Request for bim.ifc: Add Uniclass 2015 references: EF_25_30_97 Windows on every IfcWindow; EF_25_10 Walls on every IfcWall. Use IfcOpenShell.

First a look at what the model holds.

```python
import ifcopenshell

model = ifcopenshell.open("bim.ifc")
print(model.schema)
print("classifications:", [c.Name for c in model.by_type("IfcClassification")])
for ifc_class in ("IfcDoor", "IfcRoof", "IfcStair", "IfcWall", "IfcWindow"):
    print(ifc_class, len(model.by_type(ifc_class)))
```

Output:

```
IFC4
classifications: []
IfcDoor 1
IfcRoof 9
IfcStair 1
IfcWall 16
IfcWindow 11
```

```python
import ifcopenshell
import ifcopenshell.api.classification

model = ifcopenshell.open("bim.ifc")

system = ifcopenshell.api.classification.add_classification(model, classification="Uniclass 2015")

codes = {
    "IfcWindow": ("EF_25_30_97", "Windows"),
    "IfcWall": ("EF_25_10", "Walls"),
}
for ifc_class, (code, name) in codes.items():
    products = model.by_type(ifc_class)
    ifcopenshell.api.classification.add_reference(
        model, products=products, classification=system, identification=code, name=name
    )
    print(code, len(products))

model.write("bim_rev.ifc")
```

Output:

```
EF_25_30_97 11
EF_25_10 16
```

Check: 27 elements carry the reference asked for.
